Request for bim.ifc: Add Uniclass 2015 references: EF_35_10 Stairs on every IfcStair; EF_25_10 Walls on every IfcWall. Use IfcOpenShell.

First a look at what the model holds.

```python
import ifcopenshell

model = ifcopenshell.open("bim.ifc")
print(model.schema)
print("classifications:", [c.Name for c in model.by_type("IfcClassification")])
for ifc_class in ("IfcDoor", "IfcRoof", "IfcStair", "IfcWall", "IfcWindow"):
    print(ifc_class, len(model.by_type(ifc_class)))
```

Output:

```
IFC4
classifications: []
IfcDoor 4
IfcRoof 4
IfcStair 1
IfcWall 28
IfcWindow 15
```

```python
import ifcopenshell
import ifcopenshell.api.classification

model = ifcopenshell.open("bim.ifc")

system = ifcopenshell.api.classification.add_classification(model, classification="Uniclass 2015")

codes = {
    "IfcStair": ("EF_35_10", "Stairs"),
    "IfcWall": ("EF_25_10", "Walls"),
}
for ifc_class, (code, name) in codes.items():
    products = model.by_type(ifc_class)
    ifcopenshell.api.classification.add_reference(
        model, products=products, classification=system, identification=code, name=name
    )
    print(code, len(products))

model.write("bim_edited.ifc")
```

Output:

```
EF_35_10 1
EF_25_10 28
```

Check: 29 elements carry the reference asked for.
